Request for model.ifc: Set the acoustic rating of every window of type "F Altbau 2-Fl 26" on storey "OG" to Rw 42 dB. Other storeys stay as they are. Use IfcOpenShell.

First a look at what the model holds.

```python
import ifcopenshell
import ifcopenshell.util.element

model = ifcopenshell.open("model.ifc")
print(model.schema)
storey = next(s for s in model.by_type("IfcBuildingStorey") if s.Name == "OG")
windows = [e for e in ifcopenshell.util.element.get_decomposition(storey) if e.is_a("IfcWindow")]
seen = {}
for e in windows:
    element_type = ifcopenshell.util.element.get_type(e)
    key = (element_type.Name if element_type != e and element_type else None, ifcopenshell.util.element.get_pset(e, "Pset_WindowCommon", "AcousticRating"))
    seen[key] = seen.get(key, 0) + 1
for (name, value), count in sorted(seen.items(), key=str):
    print(count, "x", name, "|", value)
```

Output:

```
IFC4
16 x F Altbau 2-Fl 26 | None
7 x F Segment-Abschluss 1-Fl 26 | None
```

```python
import ifcopenshell
import ifcopenshell.api.pset
import ifcopenshell.util.element

model = ifcopenshell.open("model.ifc")

storey = next(s for s in model.by_type("IfcBuildingStorey") if s.Name == "OG")
windows = [e for e in ifcopenshell.util.element.get_decomposition(storey) if e.is_a("IfcWindow")]

count = 0
for e in windows:
    element_type = ifcopenshell.util.element.get_type(e)
    if element_type in (None, e) or element_type.Name != "F Altbau 2-Fl 26":
        continue
    # add_pset returns the element's existing set when there is one.
    pset = ifcopenshell.api.pset.add_pset(model, product=e, name="Pset_WindowCommon")
    ifcopenshell.api.pset.edit_pset(model, pset=pset, properties={"AcousticRating": "Rw 42 dB"})
    count += 1

print(count, "windows updated")

model.write("model_v2.ifc")
```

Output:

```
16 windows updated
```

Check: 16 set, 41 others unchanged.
